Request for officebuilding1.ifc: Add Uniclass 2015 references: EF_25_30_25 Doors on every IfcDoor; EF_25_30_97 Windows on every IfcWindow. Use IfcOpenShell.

First a look at what the model holds.

```python
import ifcopenshell

model = ifcopenshell.open("officebuilding1.ifc")
print(model.schema)
print("classifications:", [c.Name for c in model.by_type("IfcClassification")])
for ifc_class in ("IfcDoor", "IfcRoof", "IfcStair", "IfcWall", "IfcWindow"):
    print(ifc_class, len(model.by_type(ifc_class)))
```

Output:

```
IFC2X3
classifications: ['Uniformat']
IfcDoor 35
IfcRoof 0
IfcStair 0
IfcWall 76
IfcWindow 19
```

```python
import ifcopenshell
import ifcopenshell.api.classification

model = ifcopenshell.open("officebuilding1.ifc")

# IFC2X3 requires Source and Edition and has no link from the project to the system.
system = model.create_entity("IfcClassification", Source="NBS", Edition="2015", Name="Uniclass 2015")

codes = {
    "IfcDoor": ("EF_25_30_25", "Doors"),
    "IfcWindow": ("EF_25_30_97", "Windows"),
}
for ifc_class, (code, name) in codes.items():
    products = model.by_type(ifc_class)
    ifcopenshell.api.classification.add_reference(
        model, products=products, classification=system, identification=code, name=name
    )
    print(code, len(products))

model.write("officebuilding1_edited.ifc")
```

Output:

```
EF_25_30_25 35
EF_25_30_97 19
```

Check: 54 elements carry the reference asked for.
